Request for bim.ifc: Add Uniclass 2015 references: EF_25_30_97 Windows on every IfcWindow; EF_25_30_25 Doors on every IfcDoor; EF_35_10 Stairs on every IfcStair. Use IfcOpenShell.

First a look at what the model holds.

```python
import ifcopenshell

model = ifcopenshell.open("bim.ifc")
print(model.schema)
print("classifications:", [c.Name for c in model.by_type("IfcClassification")])
for ifc_class in ("IfcDoor", "IfcRoof", "IfcStair", "IfcWall", "IfcWindow"):
    print(ifc_class, len(model.by_type(ifc_class)))
```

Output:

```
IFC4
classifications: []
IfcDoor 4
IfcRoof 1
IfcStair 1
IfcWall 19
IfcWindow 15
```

```python
import ifcopenshell
import ifcopenshell.api.classification

model = ifcopenshell.open("bim.ifc")

system = ifcopenshell.api.classification.add_classification(model, classification="Uniclass 2015")

codes = {
    "IfcWindow": ("EF_25_30_97", "Windows"),
    "IfcDoor": ("EF_25_30_25", "Doors"),
    "IfcStair": ("EF_35_10", "Stairs"),
}
for ifc_class, (code, name) in codes.items():
    products = model.by_type(ifc_class)
    ifcopenshell.api.classification.add_reference(
        model, products=products, classification=system, identification=code, name=name
    )
    print(code, len(products))

model.write("bim_rev.ifc")
```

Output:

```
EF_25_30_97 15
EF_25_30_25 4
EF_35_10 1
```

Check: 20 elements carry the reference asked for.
